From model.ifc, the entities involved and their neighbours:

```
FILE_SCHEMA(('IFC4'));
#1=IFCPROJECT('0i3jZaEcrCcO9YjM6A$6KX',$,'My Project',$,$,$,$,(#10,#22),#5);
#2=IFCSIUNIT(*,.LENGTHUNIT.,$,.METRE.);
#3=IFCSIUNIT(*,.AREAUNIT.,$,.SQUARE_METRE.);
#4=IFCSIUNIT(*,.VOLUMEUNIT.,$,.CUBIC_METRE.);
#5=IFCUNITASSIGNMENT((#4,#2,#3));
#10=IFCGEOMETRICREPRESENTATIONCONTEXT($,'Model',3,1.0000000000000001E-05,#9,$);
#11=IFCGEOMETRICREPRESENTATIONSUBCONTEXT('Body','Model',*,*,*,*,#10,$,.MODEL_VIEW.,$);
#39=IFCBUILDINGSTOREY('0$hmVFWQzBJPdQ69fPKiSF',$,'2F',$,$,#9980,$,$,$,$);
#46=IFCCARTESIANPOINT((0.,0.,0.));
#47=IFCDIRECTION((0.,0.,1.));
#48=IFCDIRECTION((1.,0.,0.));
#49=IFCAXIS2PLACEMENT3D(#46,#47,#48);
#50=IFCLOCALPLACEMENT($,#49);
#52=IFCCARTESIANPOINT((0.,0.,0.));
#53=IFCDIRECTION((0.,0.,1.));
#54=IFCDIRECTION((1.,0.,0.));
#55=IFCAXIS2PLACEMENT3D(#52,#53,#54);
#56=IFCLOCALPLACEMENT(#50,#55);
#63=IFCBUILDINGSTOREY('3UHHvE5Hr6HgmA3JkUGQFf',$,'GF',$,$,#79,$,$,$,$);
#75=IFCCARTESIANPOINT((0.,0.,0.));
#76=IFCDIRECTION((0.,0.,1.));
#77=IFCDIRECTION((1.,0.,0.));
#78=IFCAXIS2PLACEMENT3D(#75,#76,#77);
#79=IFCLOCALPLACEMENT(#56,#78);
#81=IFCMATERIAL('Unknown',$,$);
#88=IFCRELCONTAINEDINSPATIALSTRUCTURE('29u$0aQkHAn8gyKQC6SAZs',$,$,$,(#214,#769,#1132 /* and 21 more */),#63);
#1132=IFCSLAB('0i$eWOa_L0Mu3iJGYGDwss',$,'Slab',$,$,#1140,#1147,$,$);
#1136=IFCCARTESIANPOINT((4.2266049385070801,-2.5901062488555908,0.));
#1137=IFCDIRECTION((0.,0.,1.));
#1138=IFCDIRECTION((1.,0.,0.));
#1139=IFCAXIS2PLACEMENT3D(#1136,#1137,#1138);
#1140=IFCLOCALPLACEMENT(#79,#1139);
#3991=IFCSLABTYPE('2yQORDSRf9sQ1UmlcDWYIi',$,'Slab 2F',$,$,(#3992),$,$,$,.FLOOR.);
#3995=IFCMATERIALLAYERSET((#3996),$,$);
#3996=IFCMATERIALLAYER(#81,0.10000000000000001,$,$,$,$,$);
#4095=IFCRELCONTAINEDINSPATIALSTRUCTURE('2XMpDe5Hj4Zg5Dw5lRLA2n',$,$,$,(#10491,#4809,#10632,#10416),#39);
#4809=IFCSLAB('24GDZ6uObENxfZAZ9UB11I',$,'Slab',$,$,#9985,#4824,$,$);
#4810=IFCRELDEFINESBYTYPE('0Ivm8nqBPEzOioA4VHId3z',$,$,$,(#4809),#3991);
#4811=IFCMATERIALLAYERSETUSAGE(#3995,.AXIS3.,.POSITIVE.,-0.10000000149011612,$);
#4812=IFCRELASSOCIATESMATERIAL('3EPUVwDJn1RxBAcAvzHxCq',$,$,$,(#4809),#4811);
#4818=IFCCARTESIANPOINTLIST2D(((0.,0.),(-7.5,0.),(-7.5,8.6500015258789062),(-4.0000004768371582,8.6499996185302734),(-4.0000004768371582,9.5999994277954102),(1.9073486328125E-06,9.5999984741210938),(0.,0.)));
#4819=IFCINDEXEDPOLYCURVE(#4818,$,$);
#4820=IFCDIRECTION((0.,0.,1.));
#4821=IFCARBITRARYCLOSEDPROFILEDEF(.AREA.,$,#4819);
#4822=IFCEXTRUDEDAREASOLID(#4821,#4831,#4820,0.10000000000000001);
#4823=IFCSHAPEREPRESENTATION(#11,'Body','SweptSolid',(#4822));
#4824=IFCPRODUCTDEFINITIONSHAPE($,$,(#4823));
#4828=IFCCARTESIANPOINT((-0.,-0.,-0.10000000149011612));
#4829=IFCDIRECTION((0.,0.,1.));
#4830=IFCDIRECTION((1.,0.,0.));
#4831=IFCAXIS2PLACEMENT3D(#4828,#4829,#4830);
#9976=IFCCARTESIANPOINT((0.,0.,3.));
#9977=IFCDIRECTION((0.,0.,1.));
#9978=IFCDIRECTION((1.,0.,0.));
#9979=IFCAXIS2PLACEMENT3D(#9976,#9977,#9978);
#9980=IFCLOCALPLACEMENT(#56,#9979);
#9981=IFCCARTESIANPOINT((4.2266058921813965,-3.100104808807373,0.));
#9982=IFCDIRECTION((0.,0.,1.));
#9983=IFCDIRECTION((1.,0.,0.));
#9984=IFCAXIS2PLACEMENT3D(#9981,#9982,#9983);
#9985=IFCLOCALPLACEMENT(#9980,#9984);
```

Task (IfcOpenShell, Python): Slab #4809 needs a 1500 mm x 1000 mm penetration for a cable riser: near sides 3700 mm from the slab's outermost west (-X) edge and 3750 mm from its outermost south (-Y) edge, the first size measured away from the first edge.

```python
import numpy as np
import ifcopenshell
import ifcopenshell.api.feature
import ifcopenshell.api.geometry
import ifcopenshell.api.root
import ifcopenshell.geom
import ifcopenshell.util.placement
import ifcopenshell.util.representation
import ifcopenshell.util.shape
import ifcopenshell.util.unit

model = ifcopenshell.open("model.ifc")
unit_scale = ifcopenshell.util.unit.calculate_unit_scale(model)
settings = ifcopenshell.geom.settings()


def volume(element):
    """Net volume in cubic metres, openings subtracted."""
    shape = ifcopenshell.geom.create_shape(settings, element)
    return ifcopenshell.util.shape.get_volume(shape.geometry)


slab = model.by_guid("24GDZ6uObENxfZAZ9UB11I")
before = volume(slab)

# Extent in the slab's own axes, in metres. The edges named are its -X and -Y sides.
slab_shape = ifcopenshell.geom.create_shape(settings, slab)
vertices = ifcopenshell.util.shape.get_vertices(slab_shape.geometry)
x_min, y_min, bottom = vertices.min(axis=0)
top = vertices[:, 2].max()

opening = ifcopenshell.api.root.create_entity(model, ifc_class="IfcOpeningElement", name="Cable riser opening", predefined_type="OPENING")
context = ifcopenshell.util.representation.get_context(model, "Model", "Body", "MODEL_VIEW")
width, depth = 1.5, 1
outline = [(0.0, 0.0), (width, 0.0), (width, depth), (0.0, depth), (0.0, 0.0)]
# Overshoot both faces by 50 mm so the cut is clean.
shape = ifcopenshell.api.geometry.add_slab_representation(
    model, context=context, depth=top - bottom + 0.1, polyline=outline
)
ifcopenshell.api.geometry.assign_representation(model, product=opening, representation=shape)

matrix = ifcopenshell.util.placement.get_local_placement(slab.ObjectPlacement)
matrix[:, 3] = matrix @ np.append(np.array([x_min + 3.7, y_min + 3.75, bottom - 0.05]) / unit_scale, 1.0)
ifcopenshell.api.geometry.edit_object_placement(model, product=opening, matrix=matrix, is_si=False)
ifcopenshell.api.feature.add_feature(model, feature=opening, element=slab)

after = volume(slab)

print(f"slab volume {before:.3f} -> {after:.3f} m3")

model.write("model_updated.ifc")
```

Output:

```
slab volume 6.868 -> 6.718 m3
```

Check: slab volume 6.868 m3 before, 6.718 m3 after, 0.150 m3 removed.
